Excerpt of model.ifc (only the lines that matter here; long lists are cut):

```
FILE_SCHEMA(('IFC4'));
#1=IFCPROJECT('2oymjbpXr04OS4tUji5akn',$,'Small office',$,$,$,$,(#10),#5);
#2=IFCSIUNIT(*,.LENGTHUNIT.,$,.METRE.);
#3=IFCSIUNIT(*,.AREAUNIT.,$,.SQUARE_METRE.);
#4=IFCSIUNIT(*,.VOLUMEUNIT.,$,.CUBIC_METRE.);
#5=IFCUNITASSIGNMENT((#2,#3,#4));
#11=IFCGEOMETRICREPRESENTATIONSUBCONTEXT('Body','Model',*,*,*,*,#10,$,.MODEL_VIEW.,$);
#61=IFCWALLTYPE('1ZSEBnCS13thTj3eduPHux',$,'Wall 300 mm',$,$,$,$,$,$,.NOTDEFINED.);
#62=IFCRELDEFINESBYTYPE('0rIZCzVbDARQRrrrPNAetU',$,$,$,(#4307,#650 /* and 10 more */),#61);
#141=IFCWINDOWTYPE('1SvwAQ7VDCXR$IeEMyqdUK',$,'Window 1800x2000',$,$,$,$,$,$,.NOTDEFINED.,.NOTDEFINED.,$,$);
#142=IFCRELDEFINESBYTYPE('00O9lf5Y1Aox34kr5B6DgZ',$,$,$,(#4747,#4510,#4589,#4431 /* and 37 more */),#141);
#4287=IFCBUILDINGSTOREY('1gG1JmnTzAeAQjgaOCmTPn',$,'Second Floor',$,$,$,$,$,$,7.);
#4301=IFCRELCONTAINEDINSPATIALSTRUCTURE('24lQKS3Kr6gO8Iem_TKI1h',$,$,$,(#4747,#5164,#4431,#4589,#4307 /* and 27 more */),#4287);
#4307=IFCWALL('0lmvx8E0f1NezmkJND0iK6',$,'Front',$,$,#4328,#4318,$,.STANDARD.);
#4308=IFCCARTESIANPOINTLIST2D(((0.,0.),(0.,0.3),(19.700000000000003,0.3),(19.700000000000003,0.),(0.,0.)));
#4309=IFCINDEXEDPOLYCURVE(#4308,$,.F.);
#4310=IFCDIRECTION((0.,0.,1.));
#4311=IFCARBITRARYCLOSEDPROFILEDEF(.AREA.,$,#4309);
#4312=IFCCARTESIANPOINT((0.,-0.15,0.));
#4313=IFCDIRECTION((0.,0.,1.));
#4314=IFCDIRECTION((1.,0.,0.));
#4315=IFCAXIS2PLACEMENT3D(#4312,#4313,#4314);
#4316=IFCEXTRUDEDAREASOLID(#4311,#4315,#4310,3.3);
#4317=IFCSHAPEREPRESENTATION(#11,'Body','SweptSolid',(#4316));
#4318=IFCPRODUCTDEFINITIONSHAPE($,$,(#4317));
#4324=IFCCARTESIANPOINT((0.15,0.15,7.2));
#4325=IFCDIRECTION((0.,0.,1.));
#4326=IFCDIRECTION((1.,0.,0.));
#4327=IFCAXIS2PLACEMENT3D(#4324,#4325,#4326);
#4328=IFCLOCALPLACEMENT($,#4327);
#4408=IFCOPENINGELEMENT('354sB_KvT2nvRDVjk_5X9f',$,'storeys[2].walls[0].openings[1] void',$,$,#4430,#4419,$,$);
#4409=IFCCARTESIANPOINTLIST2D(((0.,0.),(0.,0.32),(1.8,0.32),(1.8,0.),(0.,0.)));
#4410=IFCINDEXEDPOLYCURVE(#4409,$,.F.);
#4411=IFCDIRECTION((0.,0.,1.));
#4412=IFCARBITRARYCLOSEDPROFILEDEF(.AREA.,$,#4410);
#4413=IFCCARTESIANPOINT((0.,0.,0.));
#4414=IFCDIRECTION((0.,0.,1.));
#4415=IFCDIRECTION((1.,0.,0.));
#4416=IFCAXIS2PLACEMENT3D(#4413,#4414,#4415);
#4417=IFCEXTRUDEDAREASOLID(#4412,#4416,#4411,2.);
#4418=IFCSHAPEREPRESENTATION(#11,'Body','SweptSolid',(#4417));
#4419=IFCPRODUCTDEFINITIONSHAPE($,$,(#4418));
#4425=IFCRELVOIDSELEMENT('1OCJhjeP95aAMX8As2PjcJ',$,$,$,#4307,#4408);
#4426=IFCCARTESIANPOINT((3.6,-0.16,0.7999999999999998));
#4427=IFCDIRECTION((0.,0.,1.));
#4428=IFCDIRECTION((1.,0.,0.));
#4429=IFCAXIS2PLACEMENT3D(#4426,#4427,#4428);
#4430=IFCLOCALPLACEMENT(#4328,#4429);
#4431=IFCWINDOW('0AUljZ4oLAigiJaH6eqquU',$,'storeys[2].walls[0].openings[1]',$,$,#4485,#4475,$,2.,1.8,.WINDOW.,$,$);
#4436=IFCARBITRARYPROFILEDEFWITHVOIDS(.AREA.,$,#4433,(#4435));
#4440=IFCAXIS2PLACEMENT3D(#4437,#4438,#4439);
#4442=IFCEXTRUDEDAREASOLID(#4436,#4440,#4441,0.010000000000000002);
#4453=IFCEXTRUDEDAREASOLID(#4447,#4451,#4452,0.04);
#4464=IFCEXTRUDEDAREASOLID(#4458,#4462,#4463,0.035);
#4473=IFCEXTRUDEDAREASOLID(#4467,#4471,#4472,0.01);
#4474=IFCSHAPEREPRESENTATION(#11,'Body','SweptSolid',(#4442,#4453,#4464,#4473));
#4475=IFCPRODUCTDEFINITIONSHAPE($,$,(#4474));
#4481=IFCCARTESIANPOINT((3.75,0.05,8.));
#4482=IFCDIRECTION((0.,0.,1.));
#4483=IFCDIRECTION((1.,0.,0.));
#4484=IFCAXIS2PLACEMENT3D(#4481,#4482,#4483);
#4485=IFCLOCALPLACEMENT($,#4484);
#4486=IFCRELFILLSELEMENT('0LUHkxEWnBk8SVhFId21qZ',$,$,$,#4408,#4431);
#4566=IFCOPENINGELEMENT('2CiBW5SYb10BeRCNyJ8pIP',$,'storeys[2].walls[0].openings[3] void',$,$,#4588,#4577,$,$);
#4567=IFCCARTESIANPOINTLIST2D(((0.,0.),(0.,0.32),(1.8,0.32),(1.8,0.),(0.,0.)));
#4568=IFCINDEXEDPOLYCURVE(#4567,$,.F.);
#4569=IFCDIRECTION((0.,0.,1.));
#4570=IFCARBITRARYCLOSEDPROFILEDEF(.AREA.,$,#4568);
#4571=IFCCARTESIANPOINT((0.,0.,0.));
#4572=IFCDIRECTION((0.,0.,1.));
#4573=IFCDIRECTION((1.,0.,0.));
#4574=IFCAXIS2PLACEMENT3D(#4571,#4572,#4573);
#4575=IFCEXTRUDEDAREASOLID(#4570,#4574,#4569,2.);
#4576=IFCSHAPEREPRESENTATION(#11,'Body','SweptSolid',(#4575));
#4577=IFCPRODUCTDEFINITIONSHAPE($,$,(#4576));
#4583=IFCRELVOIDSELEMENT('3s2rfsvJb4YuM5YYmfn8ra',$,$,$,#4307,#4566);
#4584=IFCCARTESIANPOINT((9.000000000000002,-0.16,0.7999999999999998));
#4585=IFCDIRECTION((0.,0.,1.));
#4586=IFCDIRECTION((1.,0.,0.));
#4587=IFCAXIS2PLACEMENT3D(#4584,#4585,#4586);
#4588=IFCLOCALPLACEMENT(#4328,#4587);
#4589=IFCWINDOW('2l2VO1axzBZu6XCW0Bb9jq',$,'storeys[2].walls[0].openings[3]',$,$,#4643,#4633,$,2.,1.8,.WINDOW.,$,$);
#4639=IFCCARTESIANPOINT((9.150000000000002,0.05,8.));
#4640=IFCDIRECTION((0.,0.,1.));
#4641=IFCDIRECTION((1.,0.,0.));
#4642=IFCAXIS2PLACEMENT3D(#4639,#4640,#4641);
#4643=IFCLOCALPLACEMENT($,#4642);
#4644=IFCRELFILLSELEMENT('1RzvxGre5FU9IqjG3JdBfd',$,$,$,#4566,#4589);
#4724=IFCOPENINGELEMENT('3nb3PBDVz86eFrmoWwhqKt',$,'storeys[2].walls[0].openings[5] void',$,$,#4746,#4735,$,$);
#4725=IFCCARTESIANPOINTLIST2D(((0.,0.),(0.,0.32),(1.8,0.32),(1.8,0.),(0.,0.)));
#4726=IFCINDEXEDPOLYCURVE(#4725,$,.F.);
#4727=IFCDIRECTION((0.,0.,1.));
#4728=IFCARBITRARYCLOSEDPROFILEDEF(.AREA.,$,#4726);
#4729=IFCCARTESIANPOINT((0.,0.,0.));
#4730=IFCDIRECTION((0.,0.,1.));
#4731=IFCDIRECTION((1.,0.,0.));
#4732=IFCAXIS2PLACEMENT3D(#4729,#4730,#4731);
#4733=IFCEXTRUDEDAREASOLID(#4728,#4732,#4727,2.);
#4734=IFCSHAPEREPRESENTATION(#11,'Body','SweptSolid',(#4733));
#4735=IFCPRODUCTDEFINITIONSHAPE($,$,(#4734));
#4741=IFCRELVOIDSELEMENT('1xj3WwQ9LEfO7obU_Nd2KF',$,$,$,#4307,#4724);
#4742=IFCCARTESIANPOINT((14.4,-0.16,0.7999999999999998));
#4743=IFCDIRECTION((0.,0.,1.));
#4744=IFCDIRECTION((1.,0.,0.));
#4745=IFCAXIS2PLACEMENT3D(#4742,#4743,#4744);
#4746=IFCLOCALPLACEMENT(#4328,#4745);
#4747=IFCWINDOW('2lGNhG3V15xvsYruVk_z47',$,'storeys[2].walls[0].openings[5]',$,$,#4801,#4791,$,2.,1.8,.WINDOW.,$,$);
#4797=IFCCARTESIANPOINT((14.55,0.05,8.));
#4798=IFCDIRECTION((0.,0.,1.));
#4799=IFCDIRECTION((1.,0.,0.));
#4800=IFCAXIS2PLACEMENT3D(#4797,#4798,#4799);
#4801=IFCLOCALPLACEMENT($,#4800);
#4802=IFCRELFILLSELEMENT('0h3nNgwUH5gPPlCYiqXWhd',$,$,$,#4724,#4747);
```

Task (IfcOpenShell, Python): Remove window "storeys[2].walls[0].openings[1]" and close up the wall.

```python
import ifcopenshell
import ifcopenshell.api.feature
import ifcopenshell.api.root
import ifcopenshell.geom
import ifcopenshell.util.shape

model = ifcopenshell.open("model.ifc")
settings = ifcopenshell.geom.settings()


def volume(element):
    """Net volume in cubic metres, openings subtracted."""
    shape = ifcopenshell.geom.create_shape(settings, element)
    return ifcopenshell.util.shape.get_volume(shape.geometry)


window = model.by_guid("0AUljZ4oLAigiJaH6eqquU")
opening = window.FillsVoids[0].RelatingOpeningElement
wall = opening.VoidsElements[0].RelatingBuildingElement
before = volume(wall)

ifcopenshell.api.root.remove_product(model, product=window)
ifcopenshell.api.feature.remove_feature(model, feature=opening)

after = volume(wall)

print(f"wall volume {before:.3f} -> {after:.3f} m3")

model.write("model_edited.ifc")
```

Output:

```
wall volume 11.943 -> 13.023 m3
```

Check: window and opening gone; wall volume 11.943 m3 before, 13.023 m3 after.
